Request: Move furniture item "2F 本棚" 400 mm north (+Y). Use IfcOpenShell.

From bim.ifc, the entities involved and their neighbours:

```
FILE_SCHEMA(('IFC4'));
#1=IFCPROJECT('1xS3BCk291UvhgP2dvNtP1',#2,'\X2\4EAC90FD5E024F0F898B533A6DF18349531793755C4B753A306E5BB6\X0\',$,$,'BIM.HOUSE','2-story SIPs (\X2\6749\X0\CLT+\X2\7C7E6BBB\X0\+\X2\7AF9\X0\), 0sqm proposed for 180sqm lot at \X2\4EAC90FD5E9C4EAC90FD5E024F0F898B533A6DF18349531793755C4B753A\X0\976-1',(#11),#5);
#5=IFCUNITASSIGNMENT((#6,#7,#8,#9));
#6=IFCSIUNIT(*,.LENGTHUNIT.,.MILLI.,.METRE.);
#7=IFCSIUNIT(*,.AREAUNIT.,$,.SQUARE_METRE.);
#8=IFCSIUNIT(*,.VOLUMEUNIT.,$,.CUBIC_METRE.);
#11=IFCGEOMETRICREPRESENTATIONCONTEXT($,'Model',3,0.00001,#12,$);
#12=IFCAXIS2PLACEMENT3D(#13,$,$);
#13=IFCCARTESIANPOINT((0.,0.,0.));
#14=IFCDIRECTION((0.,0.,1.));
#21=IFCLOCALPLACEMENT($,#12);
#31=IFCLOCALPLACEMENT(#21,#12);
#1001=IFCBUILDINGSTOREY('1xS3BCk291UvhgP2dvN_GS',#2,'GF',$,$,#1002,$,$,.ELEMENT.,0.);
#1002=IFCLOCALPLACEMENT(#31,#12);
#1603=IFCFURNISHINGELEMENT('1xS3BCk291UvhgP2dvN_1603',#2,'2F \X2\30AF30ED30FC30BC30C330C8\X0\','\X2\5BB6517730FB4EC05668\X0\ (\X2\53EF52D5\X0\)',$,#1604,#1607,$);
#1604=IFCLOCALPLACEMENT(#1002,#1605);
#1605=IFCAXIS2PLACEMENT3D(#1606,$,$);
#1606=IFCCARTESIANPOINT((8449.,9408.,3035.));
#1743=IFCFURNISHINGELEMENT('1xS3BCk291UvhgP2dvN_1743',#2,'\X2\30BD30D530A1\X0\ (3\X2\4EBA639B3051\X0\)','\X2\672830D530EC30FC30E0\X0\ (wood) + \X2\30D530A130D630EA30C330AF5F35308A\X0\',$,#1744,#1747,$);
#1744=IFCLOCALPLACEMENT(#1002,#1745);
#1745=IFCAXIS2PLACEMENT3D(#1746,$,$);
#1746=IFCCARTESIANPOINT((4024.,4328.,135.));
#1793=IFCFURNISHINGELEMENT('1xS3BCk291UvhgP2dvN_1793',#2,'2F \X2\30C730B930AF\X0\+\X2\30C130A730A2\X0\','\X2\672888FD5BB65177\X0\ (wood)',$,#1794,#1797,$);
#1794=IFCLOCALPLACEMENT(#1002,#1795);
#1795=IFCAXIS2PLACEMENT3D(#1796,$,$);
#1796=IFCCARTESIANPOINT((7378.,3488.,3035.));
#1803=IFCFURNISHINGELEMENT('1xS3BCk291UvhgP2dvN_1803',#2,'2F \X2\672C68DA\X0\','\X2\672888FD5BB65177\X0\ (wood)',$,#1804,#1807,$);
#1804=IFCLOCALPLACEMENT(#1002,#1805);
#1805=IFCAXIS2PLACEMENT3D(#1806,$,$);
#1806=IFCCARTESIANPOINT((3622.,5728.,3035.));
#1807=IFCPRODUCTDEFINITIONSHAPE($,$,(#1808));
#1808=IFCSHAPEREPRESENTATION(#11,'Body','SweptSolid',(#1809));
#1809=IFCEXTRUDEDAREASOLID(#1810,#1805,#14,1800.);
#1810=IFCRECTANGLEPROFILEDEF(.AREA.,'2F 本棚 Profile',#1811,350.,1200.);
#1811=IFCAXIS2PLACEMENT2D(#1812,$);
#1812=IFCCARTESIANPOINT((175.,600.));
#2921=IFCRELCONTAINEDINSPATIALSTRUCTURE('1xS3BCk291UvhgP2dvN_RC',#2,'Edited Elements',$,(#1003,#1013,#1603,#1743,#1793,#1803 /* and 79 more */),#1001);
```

```python
import ifcopenshell
import ifcopenshell.api.geometry
import ifcopenshell.util.placement
import ifcopenshell.util.unit

model = ifcopenshell.open("bim.ifc")
unit_scale = ifcopenshell.util.unit.calculate_unit_scale(model)

item = model.by_id(1803)
matrix = ifcopenshell.util.placement.get_local_placement(item.ObjectPlacement)
matrix[1, 3] += 0.4 / unit_scale
ifcopenshell.api.geometry.edit_object_placement(model, product=item, matrix=matrix, is_si=False)

print(ifcopenshell.util.placement.get_local_placement(item.ObjectPlacement).round(3) + 0.0)

model.write("bim_updated.ifc")
```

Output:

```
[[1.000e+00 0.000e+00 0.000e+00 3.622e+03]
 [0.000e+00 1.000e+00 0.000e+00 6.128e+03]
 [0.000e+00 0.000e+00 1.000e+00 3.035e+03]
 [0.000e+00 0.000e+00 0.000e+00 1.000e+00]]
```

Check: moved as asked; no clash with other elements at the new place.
